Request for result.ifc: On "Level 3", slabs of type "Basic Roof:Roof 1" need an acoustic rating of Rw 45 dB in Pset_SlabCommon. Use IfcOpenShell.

First a look at what the model holds.

```python
import ifcopenshell
import ifcopenshell.util.element

model = ifcopenshell.open("result.ifc")
print(model.schema)
storey = next(s for s in model.by_type("IfcBuildingStorey") if s.Name == "Level 3")
slabs = [e for e in ifcopenshell.util.element.get_decomposition(storey) if e.is_a("IfcSlab")]
seen = {}
for e in slabs:
    element_type = ifcopenshell.util.element.get_type(e)
    key = (element_type.Name if element_type != e and element_type else None, ifcopenshell.util.element.get_pset(e, "Pset_SlabCommon", "AcousticRating"))
    seen[key] = seen.get(key, 0) + 1
for (name, value), count in sorted(seen.items(), key=str):
    print(count, "x", name, "|", value)
```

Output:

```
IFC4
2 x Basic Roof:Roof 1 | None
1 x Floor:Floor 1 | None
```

```python
import ifcopenshell
import ifcopenshell.api.pset
import ifcopenshell.util.element

model = ifcopenshell.open("result.ifc")

storey = next(s for s in model.by_type("IfcBuildingStorey") if s.Name == "Level 3")
slabs = [e for e in ifcopenshell.util.element.get_decomposition(storey) if e.is_a("IfcSlab")]

count = 0
for e in slabs:
    element_type = ifcopenshell.util.element.get_type(e)
    if element_type in (None, e) or element_type.Name != "Basic Roof:Roof 1":
        continue
    # add_pset returns the element's existing set when there is one.
    pset = ifcopenshell.api.pset.add_pset(model, product=e, name="Pset_SlabCommon")
    ifcopenshell.api.pset.edit_pset(model, pset=pset, properties={"AcousticRating": "Rw 45 dB"})
    count += 1

print(count, "slabs updated")

model.write("result_updated.ifc")
```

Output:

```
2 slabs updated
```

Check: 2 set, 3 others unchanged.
